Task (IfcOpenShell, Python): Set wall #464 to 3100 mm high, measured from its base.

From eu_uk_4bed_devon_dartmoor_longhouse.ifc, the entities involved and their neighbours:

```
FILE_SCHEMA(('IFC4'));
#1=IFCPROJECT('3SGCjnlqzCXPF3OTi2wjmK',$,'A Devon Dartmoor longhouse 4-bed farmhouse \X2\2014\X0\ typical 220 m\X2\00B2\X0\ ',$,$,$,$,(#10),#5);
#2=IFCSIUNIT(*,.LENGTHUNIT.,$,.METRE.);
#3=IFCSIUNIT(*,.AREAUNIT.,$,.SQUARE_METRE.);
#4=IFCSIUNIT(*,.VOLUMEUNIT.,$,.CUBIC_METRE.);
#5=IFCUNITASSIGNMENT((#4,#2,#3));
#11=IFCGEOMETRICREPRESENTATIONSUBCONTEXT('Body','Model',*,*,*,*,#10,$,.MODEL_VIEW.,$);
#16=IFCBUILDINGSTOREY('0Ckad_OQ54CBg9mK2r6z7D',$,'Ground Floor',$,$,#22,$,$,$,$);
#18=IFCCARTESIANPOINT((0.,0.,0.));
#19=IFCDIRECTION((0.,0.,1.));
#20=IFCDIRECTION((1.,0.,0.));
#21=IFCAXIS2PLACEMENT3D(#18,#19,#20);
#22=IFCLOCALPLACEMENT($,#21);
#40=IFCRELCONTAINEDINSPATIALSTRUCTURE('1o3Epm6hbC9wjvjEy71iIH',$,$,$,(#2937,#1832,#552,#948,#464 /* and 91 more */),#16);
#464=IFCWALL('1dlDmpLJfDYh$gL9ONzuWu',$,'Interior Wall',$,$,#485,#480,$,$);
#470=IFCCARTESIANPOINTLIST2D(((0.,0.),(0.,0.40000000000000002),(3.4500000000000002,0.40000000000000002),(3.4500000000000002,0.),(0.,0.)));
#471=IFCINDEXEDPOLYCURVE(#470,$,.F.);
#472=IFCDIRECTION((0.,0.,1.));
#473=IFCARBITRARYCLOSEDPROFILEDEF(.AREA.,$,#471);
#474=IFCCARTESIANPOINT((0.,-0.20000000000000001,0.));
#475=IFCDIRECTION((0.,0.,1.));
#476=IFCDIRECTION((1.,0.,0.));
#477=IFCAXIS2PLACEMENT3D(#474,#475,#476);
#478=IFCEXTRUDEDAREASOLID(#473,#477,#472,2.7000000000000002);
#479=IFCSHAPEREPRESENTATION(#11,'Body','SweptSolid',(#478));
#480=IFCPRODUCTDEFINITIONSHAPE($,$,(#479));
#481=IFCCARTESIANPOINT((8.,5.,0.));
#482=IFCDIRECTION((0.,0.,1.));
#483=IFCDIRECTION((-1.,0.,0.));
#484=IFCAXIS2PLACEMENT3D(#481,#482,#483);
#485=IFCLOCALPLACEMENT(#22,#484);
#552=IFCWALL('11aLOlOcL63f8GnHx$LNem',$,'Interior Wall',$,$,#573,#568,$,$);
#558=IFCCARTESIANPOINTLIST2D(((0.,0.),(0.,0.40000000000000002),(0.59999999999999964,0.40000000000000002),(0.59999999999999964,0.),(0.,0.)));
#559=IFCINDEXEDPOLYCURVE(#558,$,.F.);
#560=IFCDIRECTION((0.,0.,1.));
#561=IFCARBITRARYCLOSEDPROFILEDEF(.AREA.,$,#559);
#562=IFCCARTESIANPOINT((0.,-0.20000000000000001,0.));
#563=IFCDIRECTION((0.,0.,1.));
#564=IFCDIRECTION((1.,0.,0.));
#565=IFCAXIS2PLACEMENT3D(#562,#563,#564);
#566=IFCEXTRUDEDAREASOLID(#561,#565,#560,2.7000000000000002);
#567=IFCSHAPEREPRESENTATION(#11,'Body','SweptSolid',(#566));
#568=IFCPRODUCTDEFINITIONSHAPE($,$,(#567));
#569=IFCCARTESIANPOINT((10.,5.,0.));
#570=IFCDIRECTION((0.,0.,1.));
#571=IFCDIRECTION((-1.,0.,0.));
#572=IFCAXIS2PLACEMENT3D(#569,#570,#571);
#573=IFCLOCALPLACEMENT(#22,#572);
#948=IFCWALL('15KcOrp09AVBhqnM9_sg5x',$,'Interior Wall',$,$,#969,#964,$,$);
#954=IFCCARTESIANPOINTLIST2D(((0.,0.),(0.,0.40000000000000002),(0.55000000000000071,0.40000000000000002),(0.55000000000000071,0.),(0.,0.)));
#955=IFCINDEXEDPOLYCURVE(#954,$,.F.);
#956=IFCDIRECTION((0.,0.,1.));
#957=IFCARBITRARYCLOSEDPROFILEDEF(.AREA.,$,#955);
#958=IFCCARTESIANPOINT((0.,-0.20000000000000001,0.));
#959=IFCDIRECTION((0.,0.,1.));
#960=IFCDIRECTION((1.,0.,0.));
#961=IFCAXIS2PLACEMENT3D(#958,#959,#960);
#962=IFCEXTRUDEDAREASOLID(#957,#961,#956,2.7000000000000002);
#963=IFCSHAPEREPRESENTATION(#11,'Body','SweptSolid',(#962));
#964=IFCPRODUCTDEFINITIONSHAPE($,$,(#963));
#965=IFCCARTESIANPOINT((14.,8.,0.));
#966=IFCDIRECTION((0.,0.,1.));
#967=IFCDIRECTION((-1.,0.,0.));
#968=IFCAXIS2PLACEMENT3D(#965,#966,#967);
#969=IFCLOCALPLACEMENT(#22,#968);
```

```python
import ifcopenshell
import ifcopenshell.geom
import ifcopenshell.util.representation
import ifcopenshell.util.shape

model = ifcopenshell.open("eu_uk_4bed_devon_dartmoor_longhouse.ifc")
settings = ifcopenshell.geom.settings()


def volume(element):
    """Net volume in cubic metres, openings subtracted."""
    shape = ifcopenshell.geom.create_shape(settings, element)
    return ifcopenshell.util.shape.get_volume(shape.geometry)


wall = model.by_guid("1dlDmpLJfDYh$gL9ONzuWu")
before = volume(wall)

body = ifcopenshell.util.representation.get_representation(wall, "Model", "Body")
solid = body.Items[0]
old_height = solid.Depth
solid.Depth = 3.1
after = volume(wall)

print(f"height {old_height:g} -> {solid.Depth:g}, volume {before:.3f} -> {after:.3f} m3")

model.write("eu_uk_4bed_devon_dartmoor_longhouse_updated.ifc")
```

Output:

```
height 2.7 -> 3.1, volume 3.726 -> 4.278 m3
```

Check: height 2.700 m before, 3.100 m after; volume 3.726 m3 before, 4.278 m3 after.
